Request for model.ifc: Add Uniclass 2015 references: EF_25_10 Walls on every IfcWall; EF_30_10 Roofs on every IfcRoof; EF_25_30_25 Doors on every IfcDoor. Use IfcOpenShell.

First a look at what the model holds.

```python
import ifcopenshell

model = ifcopenshell.open("model.ifc")
print(model.schema)
print("classifications:", [c.Name for c in model.by_type("IfcClassification")])
for ifc_class in ("IfcDoor", "IfcRoof", "IfcStair", "IfcWall", "IfcWindow"):
    print(ifc_class, len(model.by_type(ifc_class)))
```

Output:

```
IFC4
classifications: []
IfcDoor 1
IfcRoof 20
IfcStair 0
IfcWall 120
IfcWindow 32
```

```python
import ifcopenshell
import ifcopenshell.api.classification

model = ifcopenshell.open("model.ifc")

system = ifcopenshell.api.classification.add_classification(model, classification="Uniclass 2015")

codes = {
    "IfcWall": ("EF_25_10", "Walls"),
    "IfcRoof": ("EF_30_10", "Roofs"),
    "IfcDoor": ("EF_25_30_25", "Doors"),
}
for ifc_class, (code, name) in codes.items():
    products = model.by_type(ifc_class)
    ifcopenshell.api.classification.add_reference(
        model, products=products, classification=system, identification=code, name=name
    )
    print(code, len(products))

model.write("model_edited.ifc")
```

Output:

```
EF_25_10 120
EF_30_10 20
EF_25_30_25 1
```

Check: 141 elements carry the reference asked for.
